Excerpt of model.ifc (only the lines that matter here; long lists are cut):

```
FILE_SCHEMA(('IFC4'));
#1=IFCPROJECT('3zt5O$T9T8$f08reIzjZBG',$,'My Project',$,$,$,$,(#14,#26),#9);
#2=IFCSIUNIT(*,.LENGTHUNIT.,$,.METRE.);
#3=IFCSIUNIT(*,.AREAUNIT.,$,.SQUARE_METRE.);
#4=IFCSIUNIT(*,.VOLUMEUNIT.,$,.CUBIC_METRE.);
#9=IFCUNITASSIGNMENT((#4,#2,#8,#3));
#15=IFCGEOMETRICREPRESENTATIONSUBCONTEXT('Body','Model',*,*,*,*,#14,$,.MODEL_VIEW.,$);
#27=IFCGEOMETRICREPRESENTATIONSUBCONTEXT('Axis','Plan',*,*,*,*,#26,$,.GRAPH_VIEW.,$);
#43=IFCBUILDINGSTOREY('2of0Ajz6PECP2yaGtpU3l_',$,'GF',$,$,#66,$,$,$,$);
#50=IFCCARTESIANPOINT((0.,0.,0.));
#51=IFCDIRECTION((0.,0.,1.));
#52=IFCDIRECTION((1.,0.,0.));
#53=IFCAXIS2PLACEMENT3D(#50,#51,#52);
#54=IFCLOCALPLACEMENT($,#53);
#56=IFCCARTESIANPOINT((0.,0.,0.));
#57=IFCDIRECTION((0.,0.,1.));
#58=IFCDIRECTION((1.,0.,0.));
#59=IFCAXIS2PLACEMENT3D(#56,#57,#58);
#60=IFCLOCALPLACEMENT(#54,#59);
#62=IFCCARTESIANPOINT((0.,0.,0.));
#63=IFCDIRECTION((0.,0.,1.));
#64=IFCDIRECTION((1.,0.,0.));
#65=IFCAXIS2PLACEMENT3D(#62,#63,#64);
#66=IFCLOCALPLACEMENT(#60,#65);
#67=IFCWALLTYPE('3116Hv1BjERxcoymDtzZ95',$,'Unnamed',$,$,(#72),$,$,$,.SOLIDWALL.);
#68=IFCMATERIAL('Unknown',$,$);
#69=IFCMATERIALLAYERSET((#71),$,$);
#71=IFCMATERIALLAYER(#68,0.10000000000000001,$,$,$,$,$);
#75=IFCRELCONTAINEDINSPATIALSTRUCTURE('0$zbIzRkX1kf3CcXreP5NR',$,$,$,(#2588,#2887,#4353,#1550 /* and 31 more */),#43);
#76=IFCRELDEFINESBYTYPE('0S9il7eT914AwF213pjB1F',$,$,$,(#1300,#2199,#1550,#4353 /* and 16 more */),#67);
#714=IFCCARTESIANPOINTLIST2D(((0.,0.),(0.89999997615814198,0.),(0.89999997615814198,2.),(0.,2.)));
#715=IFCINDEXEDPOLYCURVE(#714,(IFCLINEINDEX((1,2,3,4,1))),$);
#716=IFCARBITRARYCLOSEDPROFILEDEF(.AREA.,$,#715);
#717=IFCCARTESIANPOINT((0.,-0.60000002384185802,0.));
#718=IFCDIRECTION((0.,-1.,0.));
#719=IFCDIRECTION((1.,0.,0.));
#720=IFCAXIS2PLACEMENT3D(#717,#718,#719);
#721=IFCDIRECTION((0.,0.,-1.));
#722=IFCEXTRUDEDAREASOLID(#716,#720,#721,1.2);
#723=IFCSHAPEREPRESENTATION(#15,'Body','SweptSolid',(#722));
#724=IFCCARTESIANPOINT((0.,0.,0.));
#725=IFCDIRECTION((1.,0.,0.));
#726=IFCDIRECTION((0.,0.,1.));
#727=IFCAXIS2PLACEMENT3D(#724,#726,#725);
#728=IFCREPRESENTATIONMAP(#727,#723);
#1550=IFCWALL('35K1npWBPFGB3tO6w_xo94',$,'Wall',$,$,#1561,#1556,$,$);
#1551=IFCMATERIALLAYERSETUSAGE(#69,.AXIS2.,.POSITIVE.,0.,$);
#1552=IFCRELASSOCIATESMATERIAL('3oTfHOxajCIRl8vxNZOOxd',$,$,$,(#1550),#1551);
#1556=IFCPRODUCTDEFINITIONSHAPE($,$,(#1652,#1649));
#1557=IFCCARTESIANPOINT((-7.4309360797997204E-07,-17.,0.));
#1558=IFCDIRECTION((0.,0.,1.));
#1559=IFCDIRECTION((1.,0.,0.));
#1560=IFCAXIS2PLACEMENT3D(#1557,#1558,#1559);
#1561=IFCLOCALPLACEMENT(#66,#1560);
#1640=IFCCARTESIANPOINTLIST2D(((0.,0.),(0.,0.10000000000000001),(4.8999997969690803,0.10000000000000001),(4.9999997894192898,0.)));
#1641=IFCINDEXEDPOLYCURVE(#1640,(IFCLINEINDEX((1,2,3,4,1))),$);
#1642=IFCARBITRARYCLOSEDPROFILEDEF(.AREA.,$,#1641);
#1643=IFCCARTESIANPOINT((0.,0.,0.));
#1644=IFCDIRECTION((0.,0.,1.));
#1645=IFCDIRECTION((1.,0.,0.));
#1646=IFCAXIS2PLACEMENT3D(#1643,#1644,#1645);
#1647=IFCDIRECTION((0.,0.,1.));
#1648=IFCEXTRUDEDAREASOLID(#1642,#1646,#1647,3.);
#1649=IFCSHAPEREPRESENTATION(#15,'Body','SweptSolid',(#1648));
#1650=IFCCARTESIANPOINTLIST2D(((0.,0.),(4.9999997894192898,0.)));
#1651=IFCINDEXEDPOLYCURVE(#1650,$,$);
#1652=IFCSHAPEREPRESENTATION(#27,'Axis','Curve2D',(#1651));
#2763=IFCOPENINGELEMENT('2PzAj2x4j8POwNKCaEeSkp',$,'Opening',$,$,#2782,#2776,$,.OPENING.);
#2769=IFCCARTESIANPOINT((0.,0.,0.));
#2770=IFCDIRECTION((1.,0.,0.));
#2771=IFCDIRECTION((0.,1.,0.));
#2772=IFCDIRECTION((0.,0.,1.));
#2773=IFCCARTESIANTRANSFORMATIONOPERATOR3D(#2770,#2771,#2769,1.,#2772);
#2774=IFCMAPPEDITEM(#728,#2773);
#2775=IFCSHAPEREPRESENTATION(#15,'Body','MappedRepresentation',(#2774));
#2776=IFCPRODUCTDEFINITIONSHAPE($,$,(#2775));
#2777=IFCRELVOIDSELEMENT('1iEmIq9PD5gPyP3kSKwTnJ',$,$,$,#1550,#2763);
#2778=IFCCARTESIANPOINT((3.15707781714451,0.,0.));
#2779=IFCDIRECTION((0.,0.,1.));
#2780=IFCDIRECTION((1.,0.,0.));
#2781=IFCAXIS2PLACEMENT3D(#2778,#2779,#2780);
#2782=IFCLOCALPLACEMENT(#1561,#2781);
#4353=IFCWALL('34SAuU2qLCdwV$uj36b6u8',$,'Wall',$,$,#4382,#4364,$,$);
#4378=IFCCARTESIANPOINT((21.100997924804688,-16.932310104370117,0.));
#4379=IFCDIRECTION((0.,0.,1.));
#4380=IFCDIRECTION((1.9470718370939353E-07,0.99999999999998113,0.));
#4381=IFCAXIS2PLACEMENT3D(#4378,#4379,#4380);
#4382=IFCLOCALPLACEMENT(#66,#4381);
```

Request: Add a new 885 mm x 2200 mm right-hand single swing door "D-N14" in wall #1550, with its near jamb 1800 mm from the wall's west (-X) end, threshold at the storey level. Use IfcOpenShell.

```python
import numpy as np
import ifcopenshell
import ifcopenshell.api.feature
import ifcopenshell.api.geometry
import ifcopenshell.api.root
import ifcopenshell.api.spatial
import ifcopenshell.geom
import ifcopenshell.util.element
import ifcopenshell.util.placement
import ifcopenshell.util.representation
import ifcopenshell.util.shape
import ifcopenshell.util.unit

model = ifcopenshell.open("model.ifc")
unit_scale = ifcopenshell.util.unit.calculate_unit_scale(model)
settings = ifcopenshell.geom.settings()


def volume(element):
    """Net volume in cubic metres, openings subtracted."""
    shape = ifcopenshell.geom.create_shape(settings, element)
    return ifcopenshell.util.shape.get_volume(shape.geometry)


wall = model.by_id(1550)
storey = ifcopenshell.util.element.get_container(wall, ifc_class="IfcBuildingStorey")
context = ifcopenshell.util.representation.get_context(model, "Model", "Body", "MODEL_VIEW")
before = volume(wall)

width, height, from_end, sill = 0.885, 2.2, 1.8, 0.0  # metres

# The wall runs along its own X axis, and the end named is its -X end.
wall_shape = ifcopenshell.geom.create_shape(settings, wall)
x, y, z = ifcopenshell.util.shape.get_vertices(wall_shape.geometry).T
start = x.min() + from_end
face, thickness = float(y.min()), float(y.max() - y.min())
wall_matrix = ifcopenshell.util.placement.get_local_placement(wall.ObjectPlacement)
level = ifcopenshell.util.placement.get_local_placement(storey.ObjectPlacement)[2, 3]


def in_wall(x, y):
    """Placement at x, y metres in the wall's axes, at sill height."""
    matrix = wall_matrix.copy()
    matrix[:, 3] = wall_matrix @ np.array([x / unit_scale, y / unit_scale, 0.0, 1.0])
    matrix[2, 3] = level + sill / unit_scale
    return matrix


# Opening: a box that overshoots both wall faces by 50 mm.
opening = ifcopenshell.api.root.create_entity(model, ifc_class="IfcOpeningElement", predefined_type="OPENING")
box = ifcopenshell.api.geometry.add_wall_representation(
    model, context=context, length=width, height=height, thickness=thickness + 0.1
)
ifcopenshell.api.geometry.assign_representation(model, product=opening, representation=box)
ifcopenshell.api.geometry.edit_object_placement(model, product=opening, matrix=in_wall(start, face - 0.05), is_si=False)
ifcopenshell.api.feature.add_feature(model, feature=opening, element=wall)

door = ifcopenshell.api.root.create_entity(model, ifc_class="IfcDoor", name="D-N14", predefined_type="DOOR")
door.OverallWidth, door.OverallHeight = width / unit_scale, height / unit_scale
door.OperationType = "SINGLE_SWING_RIGHT"
body = ifcopenshell.api.geometry.add_door_representation(
    model,
    context=context,
    overall_width=door.OverallWidth,
    overall_height=door.OverallHeight,
    operation_type="SINGLE_SWING_RIGHT",
    lining_properties={"LiningDepth": thickness / unit_scale, "ThresholdDepth": thickness / unit_scale},
)
ifcopenshell.api.geometry.assign_representation(model, product=door, representation=body)
ifcopenshell.api.spatial.assign_container(model, products=[door], relating_structure=storey)
ifcopenshell.api.feature.add_filling(model, opening=opening, element=door)

# The lining spans the wall, so the door starts at the wall face.
ifcopenshell.api.geometry.edit_object_placement(model, product=door, matrix=in_wall(start, face), is_si=False)

after = volume(wall)

print(f"wall volume {before:.3f} -> {after:.3f} m3")

model.write("model_v2.ifc")
```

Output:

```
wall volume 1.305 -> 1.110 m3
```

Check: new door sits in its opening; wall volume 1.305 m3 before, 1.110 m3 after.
